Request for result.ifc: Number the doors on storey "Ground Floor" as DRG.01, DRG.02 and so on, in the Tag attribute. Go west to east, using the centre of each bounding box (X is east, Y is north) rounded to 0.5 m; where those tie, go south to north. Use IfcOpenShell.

First a look at what the model holds.

```python
import ifcopenshell
import ifcopenshell.util.element
import ifcopenshell.util.placement

model = ifcopenshell.open("result.ifc")
print(model.schema)
storey = next(s for s in model.by_type("IfcBuildingStorey") if s.Name == "Ground Floor")
doors = [e for e in ifcopenshell.util.element.get_decomposition(storey) if e.is_a("IfcDoor")]
for e in sorted(doors, key=lambda e: e.id()):
    origin = ifcopenshell.util.placement.get_local_placement(e.ObjectPlacement)[:3, 3]
    print(e.id(), e.Tag, e.Name, origin.round(2) + 0.0, sep=" | ")
```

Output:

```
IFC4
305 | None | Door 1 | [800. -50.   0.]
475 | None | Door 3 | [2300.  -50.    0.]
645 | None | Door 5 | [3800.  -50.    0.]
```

```python
import ifcopenshell
import ifcopenshell.geom
import ifcopenshell.util.element
import ifcopenshell.util.shape

model = ifcopenshell.open("result.ifc")
settings = ifcopenshell.geom.settings()
settings.set("use-world-coords", True)


def centre(element):
    shape = ifcopenshell.geom.create_shape(settings, element)
    return ifcopenshell.util.shape.get_bbox_centroid(shape.geometry)


storey = next(s for s in model.by_type("IfcBuildingStorey") if s.Name == "Ground Floor")
doors = [e for e in ifcopenshell.util.element.get_decomposition(storey) if e.is_a("IfcDoor")]

# Insertion points can sit at a corner or the storey origin, so sort by the geometry (in metres).
centres = {e: centre(e) for e in doors}
doors.sort(key=lambda e: (round(centres[e][0] / 0.5), centres[e][1]))

for i, e in enumerate(doors, start=1):
    number = f"DRG.{i:02d}"
    e.Tag = number
    print(e.id(), number)

model.write("result_edited.ifc")
```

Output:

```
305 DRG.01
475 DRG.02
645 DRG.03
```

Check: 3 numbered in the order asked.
